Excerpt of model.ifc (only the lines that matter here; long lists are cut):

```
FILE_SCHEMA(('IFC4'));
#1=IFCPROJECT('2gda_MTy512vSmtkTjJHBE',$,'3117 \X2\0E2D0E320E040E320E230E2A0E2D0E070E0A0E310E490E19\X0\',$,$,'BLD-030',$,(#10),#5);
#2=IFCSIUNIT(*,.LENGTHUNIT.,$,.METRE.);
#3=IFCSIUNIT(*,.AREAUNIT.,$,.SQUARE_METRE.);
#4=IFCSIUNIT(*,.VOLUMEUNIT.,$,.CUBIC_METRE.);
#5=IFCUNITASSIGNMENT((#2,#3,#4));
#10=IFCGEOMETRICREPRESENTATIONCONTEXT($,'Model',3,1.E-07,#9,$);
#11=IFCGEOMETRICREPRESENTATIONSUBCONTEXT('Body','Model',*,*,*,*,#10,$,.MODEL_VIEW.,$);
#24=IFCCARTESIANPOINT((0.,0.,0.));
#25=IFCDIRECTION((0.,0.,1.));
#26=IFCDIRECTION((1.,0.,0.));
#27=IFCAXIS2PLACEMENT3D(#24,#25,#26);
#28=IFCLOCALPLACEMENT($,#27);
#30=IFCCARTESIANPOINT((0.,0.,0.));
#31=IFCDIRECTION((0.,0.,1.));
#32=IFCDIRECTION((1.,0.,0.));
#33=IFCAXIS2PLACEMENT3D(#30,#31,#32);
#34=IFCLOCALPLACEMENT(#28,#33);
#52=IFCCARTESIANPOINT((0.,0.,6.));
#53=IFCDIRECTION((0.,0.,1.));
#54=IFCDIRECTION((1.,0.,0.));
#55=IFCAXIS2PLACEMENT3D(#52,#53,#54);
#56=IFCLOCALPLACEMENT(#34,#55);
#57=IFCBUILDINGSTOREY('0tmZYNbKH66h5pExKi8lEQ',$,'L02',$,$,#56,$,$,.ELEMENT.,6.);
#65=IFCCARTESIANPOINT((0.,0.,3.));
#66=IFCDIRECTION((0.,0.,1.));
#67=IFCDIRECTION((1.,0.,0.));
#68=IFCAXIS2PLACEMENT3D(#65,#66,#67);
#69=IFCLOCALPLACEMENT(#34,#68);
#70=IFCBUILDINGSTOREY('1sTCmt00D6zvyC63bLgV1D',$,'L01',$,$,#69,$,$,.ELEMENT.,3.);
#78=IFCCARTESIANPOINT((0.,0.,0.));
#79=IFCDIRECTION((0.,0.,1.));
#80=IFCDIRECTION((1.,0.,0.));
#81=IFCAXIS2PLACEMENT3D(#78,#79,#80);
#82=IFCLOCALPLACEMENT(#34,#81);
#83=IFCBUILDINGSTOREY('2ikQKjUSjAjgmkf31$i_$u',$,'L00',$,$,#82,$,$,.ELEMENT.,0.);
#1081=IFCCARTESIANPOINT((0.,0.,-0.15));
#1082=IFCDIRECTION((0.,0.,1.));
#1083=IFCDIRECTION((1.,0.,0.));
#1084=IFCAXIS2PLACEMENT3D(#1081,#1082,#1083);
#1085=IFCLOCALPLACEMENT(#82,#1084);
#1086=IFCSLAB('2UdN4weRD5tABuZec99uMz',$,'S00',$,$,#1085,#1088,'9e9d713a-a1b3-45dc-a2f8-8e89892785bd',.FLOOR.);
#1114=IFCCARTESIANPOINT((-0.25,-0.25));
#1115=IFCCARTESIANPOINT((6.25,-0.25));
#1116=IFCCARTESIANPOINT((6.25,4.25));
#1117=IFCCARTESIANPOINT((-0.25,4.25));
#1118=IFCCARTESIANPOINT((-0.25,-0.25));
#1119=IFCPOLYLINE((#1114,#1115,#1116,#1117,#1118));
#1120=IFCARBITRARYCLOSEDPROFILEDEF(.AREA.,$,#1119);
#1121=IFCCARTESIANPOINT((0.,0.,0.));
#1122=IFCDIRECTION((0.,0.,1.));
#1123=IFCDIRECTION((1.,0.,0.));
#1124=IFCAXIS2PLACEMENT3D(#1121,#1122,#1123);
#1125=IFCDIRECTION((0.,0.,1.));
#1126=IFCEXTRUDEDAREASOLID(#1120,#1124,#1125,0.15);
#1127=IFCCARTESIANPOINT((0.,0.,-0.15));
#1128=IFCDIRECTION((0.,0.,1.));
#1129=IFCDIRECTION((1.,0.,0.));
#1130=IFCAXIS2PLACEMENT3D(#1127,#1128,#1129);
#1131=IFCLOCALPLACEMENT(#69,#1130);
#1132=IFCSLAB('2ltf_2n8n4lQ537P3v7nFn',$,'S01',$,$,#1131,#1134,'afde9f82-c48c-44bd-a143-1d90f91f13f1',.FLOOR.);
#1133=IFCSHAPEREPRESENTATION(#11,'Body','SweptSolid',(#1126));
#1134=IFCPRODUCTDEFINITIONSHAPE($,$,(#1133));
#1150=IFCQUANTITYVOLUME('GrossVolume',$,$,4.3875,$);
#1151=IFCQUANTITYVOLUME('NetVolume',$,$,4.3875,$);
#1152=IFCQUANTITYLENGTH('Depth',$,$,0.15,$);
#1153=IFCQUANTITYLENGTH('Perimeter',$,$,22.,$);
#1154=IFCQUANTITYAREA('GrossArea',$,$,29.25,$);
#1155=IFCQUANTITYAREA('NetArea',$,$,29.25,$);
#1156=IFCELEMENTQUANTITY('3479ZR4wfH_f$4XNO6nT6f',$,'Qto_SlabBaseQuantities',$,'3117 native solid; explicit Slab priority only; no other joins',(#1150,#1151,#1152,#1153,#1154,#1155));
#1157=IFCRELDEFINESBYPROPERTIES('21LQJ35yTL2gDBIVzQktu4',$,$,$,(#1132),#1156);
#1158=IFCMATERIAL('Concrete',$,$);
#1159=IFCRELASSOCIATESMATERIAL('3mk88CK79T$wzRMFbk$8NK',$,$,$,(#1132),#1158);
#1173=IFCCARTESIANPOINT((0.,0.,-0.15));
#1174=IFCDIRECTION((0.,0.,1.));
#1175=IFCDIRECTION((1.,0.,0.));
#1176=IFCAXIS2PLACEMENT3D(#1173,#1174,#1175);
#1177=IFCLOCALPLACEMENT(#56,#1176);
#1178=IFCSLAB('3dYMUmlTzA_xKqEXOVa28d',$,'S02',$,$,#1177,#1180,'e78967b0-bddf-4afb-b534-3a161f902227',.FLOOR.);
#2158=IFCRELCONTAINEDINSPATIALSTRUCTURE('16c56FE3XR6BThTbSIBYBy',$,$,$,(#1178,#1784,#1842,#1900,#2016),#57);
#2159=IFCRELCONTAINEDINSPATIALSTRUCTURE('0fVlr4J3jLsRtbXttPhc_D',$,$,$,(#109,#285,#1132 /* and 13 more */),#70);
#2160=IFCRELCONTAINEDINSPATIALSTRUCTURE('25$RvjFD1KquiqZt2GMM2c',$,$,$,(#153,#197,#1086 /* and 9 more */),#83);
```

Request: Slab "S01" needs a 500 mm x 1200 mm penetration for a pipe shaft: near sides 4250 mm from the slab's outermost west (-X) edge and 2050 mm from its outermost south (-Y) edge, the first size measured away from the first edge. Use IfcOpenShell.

```python
import numpy as np
import ifcopenshell
import ifcopenshell.api.feature
import ifcopenshell.api.geometry
import ifcopenshell.api.pset
import ifcopenshell.api.root
import ifcopenshell.geom
import ifcopenshell.util.element
import ifcopenshell.util.placement
import ifcopenshell.util.representation
import ifcopenshell.util.shape
import ifcopenshell.util.unit

model = ifcopenshell.open("model.ifc")
unit_scale = ifcopenshell.util.unit.calculate_unit_scale(model)
area_scale = ifcopenshell.util.unit.calculate_unit_scale(model, "AREAUNIT")
volume_scale = ifcopenshell.util.unit.calculate_unit_scale(model, "VOLUMEUNIT")
settings = ifcopenshell.geom.settings()


def volume(element):
    """Net volume in cubic metres, openings subtracted."""
    shape = ifcopenshell.geom.create_shape(settings, element)
    return ifcopenshell.util.shape.get_volume(shape.geometry)


slab = model.by_guid("2ltf_2n8n4lQ537P3v7nFn")
before = volume(slab)

# Extent in the slab's own axes, in metres. The edges named are its -X and -Y sides.
slab_shape = ifcopenshell.geom.create_shape(settings, slab)
vertices = ifcopenshell.util.shape.get_vertices(slab_shape.geometry)
x_min, y_min, bottom = vertices.min(axis=0)
top = vertices[:, 2].max()

opening = ifcopenshell.api.root.create_entity(model, ifc_class="IfcOpeningElement", name="Pipe shaft opening", predefined_type="OPENING")
context = ifcopenshell.util.representation.get_context(model, "Model", "Body", "MODEL_VIEW")
width, depth = 0.5, 1.2
outline = [(0.0, 0.0), (width, 0.0), (width, depth), (0.0, depth), (0.0, 0.0)]
# Overshoot both faces by 50 mm so the cut is clean.
shape = ifcopenshell.api.geometry.add_slab_representation(
    model, context=context, depth=top - bottom + 0.1, polyline=outline
)
ifcopenshell.api.geometry.assign_representation(model, product=opening, representation=shape)

matrix = ifcopenshell.util.placement.get_local_placement(slab.ObjectPlacement)
matrix[:, 3] = matrix @ np.append(np.array([x_min + 4.25, y_min + 2.05, bottom - 0.05]) / unit_scale, 1.0)
ifcopenshell.api.geometry.edit_object_placement(model, product=opening, matrix=matrix, is_si=False)
ifcopenshell.api.feature.add_feature(model, feature=opening, element=slab)

after = volume(slab)

# Update the slab's stored quantities.
qto = model.by_id(ifcopenshell.util.element.get_pset(slab, "Qto_SlabBaseQuantities", should_inherit=False)["id"])
ifcopenshell.api.pset.edit_qto(model, qto=qto, properties={
    "NetVolume": after / volume_scale,
    "NetArea": after / (top - bottom) / area_scale,
})

print(f"slab volume {before:.3f} -> {after:.3f} m3")

model.write("model_rev.ifc")
```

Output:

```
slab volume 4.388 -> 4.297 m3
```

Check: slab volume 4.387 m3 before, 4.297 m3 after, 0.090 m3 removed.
